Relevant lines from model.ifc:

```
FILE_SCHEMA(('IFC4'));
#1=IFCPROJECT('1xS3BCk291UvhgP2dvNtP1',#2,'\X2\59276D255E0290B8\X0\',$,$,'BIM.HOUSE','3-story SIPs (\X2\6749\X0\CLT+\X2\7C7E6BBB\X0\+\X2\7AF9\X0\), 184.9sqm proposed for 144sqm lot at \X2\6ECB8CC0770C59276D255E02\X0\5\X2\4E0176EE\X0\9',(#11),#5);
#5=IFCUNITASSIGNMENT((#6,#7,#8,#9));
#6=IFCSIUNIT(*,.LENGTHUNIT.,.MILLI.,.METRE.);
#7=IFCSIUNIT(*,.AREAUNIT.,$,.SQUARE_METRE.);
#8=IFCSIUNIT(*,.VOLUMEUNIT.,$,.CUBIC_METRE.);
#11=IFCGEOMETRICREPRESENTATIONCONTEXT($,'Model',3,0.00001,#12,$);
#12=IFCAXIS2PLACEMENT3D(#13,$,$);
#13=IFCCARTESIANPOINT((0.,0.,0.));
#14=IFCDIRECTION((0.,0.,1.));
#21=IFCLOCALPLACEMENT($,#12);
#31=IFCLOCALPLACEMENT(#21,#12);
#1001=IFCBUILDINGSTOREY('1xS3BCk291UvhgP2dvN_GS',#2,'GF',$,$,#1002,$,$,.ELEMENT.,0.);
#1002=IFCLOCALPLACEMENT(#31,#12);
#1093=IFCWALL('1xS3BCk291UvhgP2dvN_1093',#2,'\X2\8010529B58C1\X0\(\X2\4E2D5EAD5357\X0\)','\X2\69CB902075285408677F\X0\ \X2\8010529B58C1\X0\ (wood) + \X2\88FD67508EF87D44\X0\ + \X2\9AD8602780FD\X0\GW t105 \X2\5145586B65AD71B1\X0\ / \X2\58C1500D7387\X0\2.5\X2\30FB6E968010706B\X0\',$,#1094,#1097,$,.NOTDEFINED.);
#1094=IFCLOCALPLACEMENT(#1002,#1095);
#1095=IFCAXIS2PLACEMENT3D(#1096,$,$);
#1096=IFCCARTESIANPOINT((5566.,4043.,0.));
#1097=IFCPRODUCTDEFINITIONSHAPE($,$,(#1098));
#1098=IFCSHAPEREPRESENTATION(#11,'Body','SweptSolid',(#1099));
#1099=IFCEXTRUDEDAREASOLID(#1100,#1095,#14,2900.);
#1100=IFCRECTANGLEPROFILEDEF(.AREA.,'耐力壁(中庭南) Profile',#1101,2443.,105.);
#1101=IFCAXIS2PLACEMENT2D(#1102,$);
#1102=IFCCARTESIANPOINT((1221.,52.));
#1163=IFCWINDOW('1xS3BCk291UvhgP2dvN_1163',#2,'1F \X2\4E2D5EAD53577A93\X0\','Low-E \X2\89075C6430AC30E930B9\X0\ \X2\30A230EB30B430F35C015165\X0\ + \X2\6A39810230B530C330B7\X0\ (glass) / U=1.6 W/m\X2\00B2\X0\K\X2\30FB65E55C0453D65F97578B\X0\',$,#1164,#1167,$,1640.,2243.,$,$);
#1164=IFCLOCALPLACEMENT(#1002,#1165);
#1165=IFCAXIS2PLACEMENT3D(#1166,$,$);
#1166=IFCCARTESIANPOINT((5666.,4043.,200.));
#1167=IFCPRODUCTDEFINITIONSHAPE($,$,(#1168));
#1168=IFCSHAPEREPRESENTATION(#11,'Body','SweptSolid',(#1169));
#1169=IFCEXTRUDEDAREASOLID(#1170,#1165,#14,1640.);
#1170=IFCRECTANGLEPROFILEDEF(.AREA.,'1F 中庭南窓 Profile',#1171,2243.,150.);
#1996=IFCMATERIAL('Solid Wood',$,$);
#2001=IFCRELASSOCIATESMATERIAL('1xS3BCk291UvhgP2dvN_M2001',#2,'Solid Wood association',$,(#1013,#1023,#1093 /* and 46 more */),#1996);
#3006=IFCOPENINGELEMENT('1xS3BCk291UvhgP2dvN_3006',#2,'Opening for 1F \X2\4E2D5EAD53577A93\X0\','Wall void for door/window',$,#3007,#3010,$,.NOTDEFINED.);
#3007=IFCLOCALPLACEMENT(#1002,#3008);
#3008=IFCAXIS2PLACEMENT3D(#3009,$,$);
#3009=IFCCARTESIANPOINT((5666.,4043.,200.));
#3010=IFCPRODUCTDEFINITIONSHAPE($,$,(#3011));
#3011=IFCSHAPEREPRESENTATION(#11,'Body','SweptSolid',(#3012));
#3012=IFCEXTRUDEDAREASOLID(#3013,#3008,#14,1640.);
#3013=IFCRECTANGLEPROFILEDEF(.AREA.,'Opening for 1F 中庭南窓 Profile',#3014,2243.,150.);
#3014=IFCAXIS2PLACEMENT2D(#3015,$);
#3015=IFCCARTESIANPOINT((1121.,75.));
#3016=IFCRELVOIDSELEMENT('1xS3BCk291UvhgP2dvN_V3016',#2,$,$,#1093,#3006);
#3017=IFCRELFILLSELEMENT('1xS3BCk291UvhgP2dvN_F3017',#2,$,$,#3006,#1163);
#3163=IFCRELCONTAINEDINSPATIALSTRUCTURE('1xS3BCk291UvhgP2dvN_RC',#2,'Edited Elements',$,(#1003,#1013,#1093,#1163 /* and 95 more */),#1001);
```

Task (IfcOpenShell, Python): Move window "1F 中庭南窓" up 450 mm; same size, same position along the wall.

```python
import numpy as np
import ifcopenshell
import ifcopenshell.api.geometry
import ifcopenshell.util.placement
import ifcopenshell.util.unit

model = ifcopenshell.open("model.ifc")
unit_scale = ifcopenshell.util.unit.calculate_unit_scale(model)

window = model.by_guid("1xS3BCk291UvhgP2dvN_1163")
opening = window.FillsVoids[0].RelatingOpeningElement
dz = 450.0

shift = np.array([0.0, 0.0, dz])
# The window is not placed relative to its opening, so move both.
for product in (opening, window):
    matrix = ifcopenshell.util.placement.get_local_placement(product.ObjectPlacement)
    matrix[:3, 3] += shift
    ifcopenshell.api.geometry.edit_object_placement(model, product=product, matrix=matrix, is_si=False)

print(f"moved by {dz * unit_scale:+.3f} m")

model.write("model_updated.ifc")
```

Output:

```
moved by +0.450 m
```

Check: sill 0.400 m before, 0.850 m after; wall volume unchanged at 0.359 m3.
